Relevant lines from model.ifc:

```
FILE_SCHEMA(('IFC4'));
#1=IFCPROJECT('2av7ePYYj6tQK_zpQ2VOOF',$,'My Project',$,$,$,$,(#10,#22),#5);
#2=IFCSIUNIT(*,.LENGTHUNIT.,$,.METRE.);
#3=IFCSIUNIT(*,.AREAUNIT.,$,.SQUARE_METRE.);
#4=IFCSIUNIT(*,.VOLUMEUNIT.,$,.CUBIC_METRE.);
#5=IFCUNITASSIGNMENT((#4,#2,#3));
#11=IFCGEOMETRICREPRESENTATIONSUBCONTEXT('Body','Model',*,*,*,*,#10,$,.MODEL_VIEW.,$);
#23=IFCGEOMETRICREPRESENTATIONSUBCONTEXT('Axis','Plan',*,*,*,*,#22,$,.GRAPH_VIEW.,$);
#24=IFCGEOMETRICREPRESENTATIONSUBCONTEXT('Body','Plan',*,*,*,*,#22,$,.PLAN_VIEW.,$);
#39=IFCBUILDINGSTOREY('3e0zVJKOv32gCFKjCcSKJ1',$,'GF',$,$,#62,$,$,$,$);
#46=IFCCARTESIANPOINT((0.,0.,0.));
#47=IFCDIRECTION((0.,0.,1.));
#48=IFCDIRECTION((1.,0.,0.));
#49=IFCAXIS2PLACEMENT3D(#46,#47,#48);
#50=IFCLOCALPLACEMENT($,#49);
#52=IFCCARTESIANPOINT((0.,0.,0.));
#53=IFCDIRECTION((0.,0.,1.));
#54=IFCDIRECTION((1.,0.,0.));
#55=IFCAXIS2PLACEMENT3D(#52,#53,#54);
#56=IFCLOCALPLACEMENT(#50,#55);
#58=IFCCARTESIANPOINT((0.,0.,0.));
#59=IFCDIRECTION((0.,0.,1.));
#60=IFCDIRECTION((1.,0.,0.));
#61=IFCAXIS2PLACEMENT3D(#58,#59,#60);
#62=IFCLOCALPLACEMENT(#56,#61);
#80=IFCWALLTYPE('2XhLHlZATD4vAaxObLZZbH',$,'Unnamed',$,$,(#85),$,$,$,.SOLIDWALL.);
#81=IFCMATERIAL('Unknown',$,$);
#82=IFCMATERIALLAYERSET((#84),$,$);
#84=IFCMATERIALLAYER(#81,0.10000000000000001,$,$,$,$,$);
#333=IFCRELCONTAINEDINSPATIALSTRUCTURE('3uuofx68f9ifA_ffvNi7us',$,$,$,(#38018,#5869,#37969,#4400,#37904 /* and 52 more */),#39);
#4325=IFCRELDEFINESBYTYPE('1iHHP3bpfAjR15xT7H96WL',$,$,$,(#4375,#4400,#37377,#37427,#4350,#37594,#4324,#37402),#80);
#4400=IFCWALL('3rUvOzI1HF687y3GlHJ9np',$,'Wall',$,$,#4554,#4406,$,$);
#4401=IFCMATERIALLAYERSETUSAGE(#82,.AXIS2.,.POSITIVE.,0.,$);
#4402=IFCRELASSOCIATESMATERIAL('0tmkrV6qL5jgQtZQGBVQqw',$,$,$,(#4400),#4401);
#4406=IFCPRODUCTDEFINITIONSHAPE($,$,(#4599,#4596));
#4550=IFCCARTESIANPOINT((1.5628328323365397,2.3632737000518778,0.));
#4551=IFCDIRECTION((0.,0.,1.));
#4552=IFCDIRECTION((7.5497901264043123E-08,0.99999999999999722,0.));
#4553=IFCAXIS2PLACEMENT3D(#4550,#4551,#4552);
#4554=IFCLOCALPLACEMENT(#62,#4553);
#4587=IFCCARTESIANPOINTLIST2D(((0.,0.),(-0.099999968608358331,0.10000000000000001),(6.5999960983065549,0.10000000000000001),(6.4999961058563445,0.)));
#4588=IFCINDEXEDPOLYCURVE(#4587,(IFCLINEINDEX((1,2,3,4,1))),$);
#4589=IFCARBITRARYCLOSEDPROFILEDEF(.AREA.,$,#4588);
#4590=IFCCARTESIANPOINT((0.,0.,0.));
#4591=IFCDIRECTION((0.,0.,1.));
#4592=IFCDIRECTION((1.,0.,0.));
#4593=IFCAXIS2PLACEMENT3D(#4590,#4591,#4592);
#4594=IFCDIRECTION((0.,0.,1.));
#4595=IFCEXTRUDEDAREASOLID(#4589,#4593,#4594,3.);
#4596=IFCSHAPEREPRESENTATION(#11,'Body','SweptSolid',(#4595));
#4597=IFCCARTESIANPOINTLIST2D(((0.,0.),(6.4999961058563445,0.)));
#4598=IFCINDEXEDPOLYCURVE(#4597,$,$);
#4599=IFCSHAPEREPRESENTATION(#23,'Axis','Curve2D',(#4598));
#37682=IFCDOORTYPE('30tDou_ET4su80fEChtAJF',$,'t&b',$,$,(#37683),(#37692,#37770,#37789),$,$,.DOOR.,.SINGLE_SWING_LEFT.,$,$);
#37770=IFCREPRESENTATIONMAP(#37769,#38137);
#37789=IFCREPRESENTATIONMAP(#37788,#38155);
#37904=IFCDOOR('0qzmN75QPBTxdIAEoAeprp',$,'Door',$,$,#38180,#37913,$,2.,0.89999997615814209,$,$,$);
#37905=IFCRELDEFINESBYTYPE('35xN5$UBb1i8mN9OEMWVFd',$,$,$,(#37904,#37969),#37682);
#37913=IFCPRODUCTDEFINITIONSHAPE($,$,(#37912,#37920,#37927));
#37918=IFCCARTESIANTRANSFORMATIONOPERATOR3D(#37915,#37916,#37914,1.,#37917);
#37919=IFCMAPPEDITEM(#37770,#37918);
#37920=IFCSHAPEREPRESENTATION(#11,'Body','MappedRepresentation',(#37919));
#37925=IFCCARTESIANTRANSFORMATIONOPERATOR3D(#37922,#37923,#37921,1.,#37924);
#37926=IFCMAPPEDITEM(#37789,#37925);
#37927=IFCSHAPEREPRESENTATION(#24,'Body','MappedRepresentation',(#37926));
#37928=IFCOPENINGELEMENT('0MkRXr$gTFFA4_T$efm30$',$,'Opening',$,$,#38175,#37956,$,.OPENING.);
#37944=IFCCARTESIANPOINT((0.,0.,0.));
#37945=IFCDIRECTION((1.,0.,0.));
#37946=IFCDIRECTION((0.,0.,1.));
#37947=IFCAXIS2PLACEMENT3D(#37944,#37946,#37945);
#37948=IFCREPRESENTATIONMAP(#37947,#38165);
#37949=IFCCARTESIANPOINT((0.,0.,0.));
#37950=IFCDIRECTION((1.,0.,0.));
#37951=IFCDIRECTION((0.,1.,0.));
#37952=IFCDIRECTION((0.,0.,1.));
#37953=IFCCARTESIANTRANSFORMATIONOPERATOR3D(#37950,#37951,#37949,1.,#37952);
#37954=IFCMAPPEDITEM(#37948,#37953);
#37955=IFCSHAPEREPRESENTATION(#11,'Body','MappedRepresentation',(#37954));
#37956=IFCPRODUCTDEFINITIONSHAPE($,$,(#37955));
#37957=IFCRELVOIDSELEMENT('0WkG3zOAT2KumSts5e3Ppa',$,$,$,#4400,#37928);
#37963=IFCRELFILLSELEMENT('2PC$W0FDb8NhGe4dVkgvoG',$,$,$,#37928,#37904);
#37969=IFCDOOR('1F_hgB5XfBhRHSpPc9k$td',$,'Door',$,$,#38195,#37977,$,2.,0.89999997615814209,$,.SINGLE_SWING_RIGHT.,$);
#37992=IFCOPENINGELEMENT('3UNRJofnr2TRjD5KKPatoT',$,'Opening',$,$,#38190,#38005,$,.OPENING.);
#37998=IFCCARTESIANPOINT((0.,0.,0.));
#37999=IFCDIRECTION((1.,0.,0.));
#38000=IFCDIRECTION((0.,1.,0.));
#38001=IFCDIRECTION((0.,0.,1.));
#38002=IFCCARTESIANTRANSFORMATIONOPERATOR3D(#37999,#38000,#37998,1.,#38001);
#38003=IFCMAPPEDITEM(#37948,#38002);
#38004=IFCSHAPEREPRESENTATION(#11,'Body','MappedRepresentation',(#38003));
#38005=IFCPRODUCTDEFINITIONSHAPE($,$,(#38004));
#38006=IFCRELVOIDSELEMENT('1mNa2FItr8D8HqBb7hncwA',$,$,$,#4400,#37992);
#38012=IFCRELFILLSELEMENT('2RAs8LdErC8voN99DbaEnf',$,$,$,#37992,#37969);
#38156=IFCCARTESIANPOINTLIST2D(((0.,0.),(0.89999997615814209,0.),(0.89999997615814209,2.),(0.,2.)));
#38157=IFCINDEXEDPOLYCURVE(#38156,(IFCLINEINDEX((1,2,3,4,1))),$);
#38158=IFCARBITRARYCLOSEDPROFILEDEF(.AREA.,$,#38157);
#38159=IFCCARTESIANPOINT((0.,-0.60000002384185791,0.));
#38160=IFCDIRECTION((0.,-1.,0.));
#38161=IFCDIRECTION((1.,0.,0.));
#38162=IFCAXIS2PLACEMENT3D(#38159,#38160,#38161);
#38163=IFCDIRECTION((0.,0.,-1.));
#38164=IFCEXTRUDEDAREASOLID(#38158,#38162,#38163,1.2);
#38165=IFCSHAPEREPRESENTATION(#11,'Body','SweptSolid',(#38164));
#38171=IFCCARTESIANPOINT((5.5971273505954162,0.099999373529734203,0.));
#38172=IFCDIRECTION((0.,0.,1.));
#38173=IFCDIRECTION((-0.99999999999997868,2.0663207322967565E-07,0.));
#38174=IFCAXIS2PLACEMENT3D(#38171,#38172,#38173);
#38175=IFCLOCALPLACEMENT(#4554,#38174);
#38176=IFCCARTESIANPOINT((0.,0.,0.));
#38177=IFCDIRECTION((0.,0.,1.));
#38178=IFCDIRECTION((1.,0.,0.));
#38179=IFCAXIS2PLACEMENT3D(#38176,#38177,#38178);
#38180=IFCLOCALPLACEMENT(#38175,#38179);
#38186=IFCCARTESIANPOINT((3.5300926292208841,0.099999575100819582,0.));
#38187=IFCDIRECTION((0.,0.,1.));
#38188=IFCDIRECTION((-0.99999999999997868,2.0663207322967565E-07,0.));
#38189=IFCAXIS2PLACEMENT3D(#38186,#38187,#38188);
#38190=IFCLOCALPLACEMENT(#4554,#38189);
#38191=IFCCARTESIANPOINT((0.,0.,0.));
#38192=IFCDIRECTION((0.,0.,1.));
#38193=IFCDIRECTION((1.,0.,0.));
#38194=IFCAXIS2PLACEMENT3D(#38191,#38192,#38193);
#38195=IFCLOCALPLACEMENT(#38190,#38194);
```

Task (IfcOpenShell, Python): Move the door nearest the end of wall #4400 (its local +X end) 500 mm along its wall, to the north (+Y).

```python
import ifcopenshell
import ifcopenshell.api.geometry
import ifcopenshell.util.placement

model = ifcopenshell.open("model.ifc")

door = model.by_id(37904)
opening = door.FillsVoids[0].RelatingOpeningElement
wall = opening.VoidsElements[0].RelatingBuildingElement

wall_matrix = ifcopenshell.util.placement.get_local_placement(wall.ObjectPlacement)
shift = wall_matrix[:3, 0] * 0.5
before = ifcopenshell.util.placement.get_local_placement(door.ObjectPlacement)[:3, 3].copy()

# The door is placed relative to its opening, so it follows when the opening moves.
matrix = ifcopenshell.util.placement.get_local_placement(opening.ObjectPlacement)
matrix[:3, 3] += shift
ifcopenshell.api.geometry.edit_object_placement(
    model, product=opening, matrix=matrix, is_si=False, should_transform_children=True
)

after = ifcopenshell.util.placement.get_local_placement(door.ObjectPlacement)[:3, 3]
print("door moved by", (after - before).round(3) + 0.0)

model.write("model_v2.ifc")
```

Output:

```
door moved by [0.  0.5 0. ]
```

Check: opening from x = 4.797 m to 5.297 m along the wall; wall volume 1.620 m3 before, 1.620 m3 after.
